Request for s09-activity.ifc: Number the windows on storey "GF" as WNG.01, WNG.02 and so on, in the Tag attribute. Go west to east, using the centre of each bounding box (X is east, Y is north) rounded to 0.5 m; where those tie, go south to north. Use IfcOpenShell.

First a look at what the model holds.

```python
import ifcopenshell
import ifcopenshell.util.element
import ifcopenshell.util.placement

model = ifcopenshell.open("s09-activity.ifc")
print(model.schema)
storey = next(s for s in model.by_type("IfcBuildingStorey") if s.Name == "GF")
windows = [e for e in ifcopenshell.util.element.get_decomposition(storey) if e.is_a("IfcWindow")]
for e in sorted(windows, key=lambda e: e.id()):
    origin = ifcopenshell.util.placement.get_local_placement(e.ObjectPlacement)[:3, 3]
    print(e.id(), e.Tag, e.Name, origin.round(2) + 0.0, sep=" | ")
```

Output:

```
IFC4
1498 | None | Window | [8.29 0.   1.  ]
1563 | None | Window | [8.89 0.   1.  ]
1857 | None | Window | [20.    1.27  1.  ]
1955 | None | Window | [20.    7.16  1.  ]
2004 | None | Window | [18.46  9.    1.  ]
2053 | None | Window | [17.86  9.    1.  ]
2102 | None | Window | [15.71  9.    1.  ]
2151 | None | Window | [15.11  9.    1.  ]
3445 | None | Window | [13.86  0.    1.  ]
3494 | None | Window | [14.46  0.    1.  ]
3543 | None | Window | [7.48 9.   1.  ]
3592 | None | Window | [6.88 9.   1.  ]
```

```python
import ifcopenshell
import ifcopenshell.geom
import ifcopenshell.util.element
import ifcopenshell.util.shape

model = ifcopenshell.open("s09-activity.ifc")
settings = ifcopenshell.geom.settings()
settings.set("use-world-coords", True)


def centre(element):
    shape = ifcopenshell.geom.create_shape(settings, element)
    return ifcopenshell.util.shape.get_bbox_centroid(shape.geometry)


storey = next(s for s in model.by_type("IfcBuildingStorey") if s.Name == "GF")
windows = [e for e in ifcopenshell.util.element.get_decomposition(storey) if e.is_a("IfcWindow")]

# Insertion points can sit at a corner or the storey origin, so sort by the geometry (in metres).
centres = {e: centre(e) for e in windows}
windows.sort(key=lambda e: (round(centres[e][0] / 0.5), centres[e][1]))

for i, e in enumerate(windows, start=1):
    number = f"WNG.{i:02d}"
    e.Tag = number
    print(e.id(), number)

model.write("s09-activity-out.ifc")
```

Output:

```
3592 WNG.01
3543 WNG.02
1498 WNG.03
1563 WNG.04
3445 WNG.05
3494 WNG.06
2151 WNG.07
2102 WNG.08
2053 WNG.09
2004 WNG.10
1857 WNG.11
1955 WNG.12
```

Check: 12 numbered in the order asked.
